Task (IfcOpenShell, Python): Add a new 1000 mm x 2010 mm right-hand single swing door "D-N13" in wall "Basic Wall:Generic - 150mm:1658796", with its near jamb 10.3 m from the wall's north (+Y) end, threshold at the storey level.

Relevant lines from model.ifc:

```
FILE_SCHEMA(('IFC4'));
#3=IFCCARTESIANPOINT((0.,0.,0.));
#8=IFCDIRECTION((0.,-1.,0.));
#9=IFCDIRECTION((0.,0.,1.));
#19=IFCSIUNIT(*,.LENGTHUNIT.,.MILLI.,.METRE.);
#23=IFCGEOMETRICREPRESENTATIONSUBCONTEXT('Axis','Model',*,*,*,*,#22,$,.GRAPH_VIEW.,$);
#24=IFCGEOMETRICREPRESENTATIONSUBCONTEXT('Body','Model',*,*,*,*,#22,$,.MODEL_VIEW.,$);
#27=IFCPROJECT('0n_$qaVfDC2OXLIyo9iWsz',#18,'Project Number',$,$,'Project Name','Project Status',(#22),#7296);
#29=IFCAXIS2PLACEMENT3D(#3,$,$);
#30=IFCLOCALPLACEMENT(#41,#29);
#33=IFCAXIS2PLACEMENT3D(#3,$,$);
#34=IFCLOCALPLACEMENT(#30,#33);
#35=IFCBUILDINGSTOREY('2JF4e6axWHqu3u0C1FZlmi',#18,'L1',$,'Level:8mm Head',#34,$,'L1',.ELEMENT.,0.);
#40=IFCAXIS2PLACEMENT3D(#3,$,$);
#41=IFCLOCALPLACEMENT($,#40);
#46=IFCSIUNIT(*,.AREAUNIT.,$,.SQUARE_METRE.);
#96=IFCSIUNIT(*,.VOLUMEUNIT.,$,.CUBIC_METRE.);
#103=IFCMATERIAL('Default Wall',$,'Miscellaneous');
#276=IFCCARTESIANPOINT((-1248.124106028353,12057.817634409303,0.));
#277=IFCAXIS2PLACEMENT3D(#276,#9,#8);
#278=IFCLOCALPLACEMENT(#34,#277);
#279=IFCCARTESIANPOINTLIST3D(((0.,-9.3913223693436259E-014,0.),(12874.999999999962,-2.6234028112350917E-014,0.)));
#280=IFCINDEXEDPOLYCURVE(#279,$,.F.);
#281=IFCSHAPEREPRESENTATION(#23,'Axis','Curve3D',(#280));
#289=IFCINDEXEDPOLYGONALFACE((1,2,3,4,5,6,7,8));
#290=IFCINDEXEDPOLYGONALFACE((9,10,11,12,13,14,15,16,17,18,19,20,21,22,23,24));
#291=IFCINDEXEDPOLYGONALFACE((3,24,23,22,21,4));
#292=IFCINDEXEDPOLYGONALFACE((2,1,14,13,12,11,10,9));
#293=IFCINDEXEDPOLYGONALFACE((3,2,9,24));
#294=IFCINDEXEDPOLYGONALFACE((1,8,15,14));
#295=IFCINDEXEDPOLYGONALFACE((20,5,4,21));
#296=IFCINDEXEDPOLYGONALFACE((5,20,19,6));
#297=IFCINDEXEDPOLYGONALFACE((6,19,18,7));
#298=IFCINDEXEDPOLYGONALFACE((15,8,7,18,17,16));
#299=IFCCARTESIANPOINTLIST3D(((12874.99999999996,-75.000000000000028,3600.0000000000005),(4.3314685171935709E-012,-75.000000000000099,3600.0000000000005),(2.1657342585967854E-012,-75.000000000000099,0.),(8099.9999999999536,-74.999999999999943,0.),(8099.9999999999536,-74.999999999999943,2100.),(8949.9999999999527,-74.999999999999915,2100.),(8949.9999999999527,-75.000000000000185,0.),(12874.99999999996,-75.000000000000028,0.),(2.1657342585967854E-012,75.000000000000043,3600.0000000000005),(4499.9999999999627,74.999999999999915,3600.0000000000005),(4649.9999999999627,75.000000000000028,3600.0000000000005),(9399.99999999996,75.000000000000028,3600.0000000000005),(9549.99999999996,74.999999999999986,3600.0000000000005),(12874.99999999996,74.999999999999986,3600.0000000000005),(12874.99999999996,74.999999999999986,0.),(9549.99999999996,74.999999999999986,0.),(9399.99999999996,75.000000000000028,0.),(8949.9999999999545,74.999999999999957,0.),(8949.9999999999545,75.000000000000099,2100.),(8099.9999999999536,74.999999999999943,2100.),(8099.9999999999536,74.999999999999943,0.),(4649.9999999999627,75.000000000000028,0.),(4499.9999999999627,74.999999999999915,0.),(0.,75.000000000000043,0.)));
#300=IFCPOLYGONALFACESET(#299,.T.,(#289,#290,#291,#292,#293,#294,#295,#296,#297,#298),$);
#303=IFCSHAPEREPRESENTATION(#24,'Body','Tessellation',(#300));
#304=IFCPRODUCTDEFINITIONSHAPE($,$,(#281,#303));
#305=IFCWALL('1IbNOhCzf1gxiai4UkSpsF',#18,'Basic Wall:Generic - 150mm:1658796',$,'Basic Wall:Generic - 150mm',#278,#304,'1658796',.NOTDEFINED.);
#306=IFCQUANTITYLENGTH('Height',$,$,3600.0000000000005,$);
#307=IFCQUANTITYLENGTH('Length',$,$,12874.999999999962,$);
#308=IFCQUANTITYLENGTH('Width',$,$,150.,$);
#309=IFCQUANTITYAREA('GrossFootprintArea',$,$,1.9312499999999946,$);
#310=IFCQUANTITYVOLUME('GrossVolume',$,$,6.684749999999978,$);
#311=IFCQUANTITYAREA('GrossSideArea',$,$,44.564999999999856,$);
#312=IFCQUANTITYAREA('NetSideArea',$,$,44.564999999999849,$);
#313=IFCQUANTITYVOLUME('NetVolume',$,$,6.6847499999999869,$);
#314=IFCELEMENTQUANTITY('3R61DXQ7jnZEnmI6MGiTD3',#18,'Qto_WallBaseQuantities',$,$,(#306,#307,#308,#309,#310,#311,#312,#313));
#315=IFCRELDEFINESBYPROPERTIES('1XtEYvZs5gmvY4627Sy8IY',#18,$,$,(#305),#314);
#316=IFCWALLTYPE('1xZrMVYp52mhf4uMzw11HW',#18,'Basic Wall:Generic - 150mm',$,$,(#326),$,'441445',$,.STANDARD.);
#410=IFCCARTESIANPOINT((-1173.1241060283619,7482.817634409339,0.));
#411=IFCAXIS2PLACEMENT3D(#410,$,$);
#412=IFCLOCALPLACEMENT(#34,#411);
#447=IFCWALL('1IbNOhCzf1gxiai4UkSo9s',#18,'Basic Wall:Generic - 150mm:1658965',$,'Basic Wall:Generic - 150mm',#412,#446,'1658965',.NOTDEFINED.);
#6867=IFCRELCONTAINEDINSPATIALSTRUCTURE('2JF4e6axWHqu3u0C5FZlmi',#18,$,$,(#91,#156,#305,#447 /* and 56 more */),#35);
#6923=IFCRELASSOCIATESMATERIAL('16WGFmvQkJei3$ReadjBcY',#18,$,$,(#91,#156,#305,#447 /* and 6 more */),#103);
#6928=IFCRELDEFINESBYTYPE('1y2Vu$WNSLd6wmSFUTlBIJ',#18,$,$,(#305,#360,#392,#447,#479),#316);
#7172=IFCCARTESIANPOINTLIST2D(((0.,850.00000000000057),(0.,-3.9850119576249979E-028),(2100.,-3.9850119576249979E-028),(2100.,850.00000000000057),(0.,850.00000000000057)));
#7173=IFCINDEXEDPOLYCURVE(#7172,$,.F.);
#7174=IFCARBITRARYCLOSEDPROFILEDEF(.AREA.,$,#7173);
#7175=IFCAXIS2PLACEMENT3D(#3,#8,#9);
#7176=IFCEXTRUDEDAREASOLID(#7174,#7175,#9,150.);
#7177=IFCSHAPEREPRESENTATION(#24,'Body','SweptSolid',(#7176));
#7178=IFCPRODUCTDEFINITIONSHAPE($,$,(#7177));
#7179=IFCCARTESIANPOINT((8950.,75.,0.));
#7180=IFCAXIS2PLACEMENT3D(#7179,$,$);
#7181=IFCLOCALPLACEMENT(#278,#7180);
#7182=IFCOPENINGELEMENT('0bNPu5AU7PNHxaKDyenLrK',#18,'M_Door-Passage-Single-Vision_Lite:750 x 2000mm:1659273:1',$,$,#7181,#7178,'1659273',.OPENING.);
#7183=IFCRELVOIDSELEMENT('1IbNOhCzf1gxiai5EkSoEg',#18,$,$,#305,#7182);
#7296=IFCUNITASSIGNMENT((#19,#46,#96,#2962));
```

```python
import numpy as np
import ifcopenshell
import ifcopenshell.api.feature
import ifcopenshell.api.geometry
import ifcopenshell.api.pset
import ifcopenshell.api.root
import ifcopenshell.api.spatial
import ifcopenshell.geom
import ifcopenshell.util.element
import ifcopenshell.util.placement
import ifcopenshell.util.representation
import ifcopenshell.util.shape
import ifcopenshell.util.unit

model = ifcopenshell.open("model.ifc")
unit_scale = ifcopenshell.util.unit.calculate_unit_scale(model)
area_scale = ifcopenshell.util.unit.calculate_unit_scale(model, "AREAUNIT")
volume_scale = ifcopenshell.util.unit.calculate_unit_scale(model, "VOLUMEUNIT")
settings = ifcopenshell.geom.settings()


def volume(element):
    """Net volume in cubic metres, openings subtracted."""
    shape = ifcopenshell.geom.create_shape(settings, element)
    return ifcopenshell.util.shape.get_volume(shape.geometry)


wall = model.by_guid("1IbNOhCzf1gxiai4UkSpsF")
storey = ifcopenshell.util.element.get_container(wall, ifc_class="IfcBuildingStorey")
context = ifcopenshell.util.representation.get_context(model, "Model", "Body", "MODEL_VIEW")
before = volume(wall)

width, height, from_end, sill = 1, 2.01, 10.3, 0.0  # metres

# The wall runs along its own X axis, and the end named is its -X end.
wall_shape = ifcopenshell.geom.create_shape(settings, wall)
x, y, z = ifcopenshell.util.shape.get_vertices(wall_shape.geometry).T
start = x.min() + from_end
face, thickness = float(y.min()), float(y.max() - y.min())
wall_matrix = ifcopenshell.util.placement.get_local_placement(wall.ObjectPlacement)
level = ifcopenshell.util.placement.get_local_placement(storey.ObjectPlacement)[2, 3]


def in_wall(x, y):
    """Placement at x, y metres in the wall's axes, at sill height."""
    matrix = wall_matrix.copy()
    matrix[:, 3] = wall_matrix @ np.array([x / unit_scale, y / unit_scale, 0.0, 1.0])
    matrix[2, 3] = level + sill / unit_scale
    return matrix


# Opening: a box that overshoots both wall faces by 50 mm.
opening = ifcopenshell.api.root.create_entity(model, ifc_class="IfcOpeningElement", predefined_type="OPENING")
box = ifcopenshell.api.geometry.add_wall_representation(
    model, context=context, length=width, height=height, thickness=thickness + 0.1
)
ifcopenshell.api.geometry.assign_representation(model, product=opening, representation=box)
ifcopenshell.api.geometry.edit_object_placement(model, product=opening, matrix=in_wall(start, face - 0.05), is_si=False)
ifcopenshell.api.feature.add_feature(model, feature=opening, element=wall)

door = ifcopenshell.api.root.create_entity(model, ifc_class="IfcDoor", name="D-N13", predefined_type="DOOR")
door.OverallWidth, door.OverallHeight = width / unit_scale, height / unit_scale
door.OperationType = "SINGLE_SWING_RIGHT"
body = ifcopenshell.api.geometry.add_door_representation(
    model,
    context=context,
    overall_width=door.OverallWidth,
    overall_height=door.OverallHeight,
    operation_type="SINGLE_SWING_RIGHT",
    lining_properties={"LiningDepth": thickness / unit_scale, "ThresholdDepth": thickness / unit_scale},
)
ifcopenshell.api.geometry.assign_representation(model, product=door, representation=body)
ifcopenshell.api.spatial.assign_container(model, products=[door], relating_structure=storey)
ifcopenshell.api.feature.add_filling(model, opening=opening, element=door)

# The lining spans the wall, so the door starts at the wall face.
ifcopenshell.api.geometry.edit_object_placement(model, product=door, matrix=in_wall(start, face), is_si=False)

after = volume(wall)

# Update the wall's stored quantities.
qto = model.by_id(ifcopenshell.util.element.get_pset(wall, "Qto_WallBaseQuantities", should_inherit=False)["id"])
ifcopenshell.api.pset.edit_qto(model, qto=qto, properties={
    "NetSideArea": after / thickness / area_scale,
    "NetVolume": after / volume_scale,
})

print(f"wall volume {before:.3f} -> {after:.3f} m3")

model.write("model_v2.ifc")
```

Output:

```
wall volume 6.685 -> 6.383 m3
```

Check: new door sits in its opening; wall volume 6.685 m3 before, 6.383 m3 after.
